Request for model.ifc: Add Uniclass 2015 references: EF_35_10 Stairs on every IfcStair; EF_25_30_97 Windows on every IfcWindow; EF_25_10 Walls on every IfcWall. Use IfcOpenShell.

First a look at what the model holds.

```python
import ifcopenshell

model = ifcopenshell.open("model.ifc")
print(model.schema)
print("classifications:", [c.Name for c in model.by_type("IfcClassification")])
for ifc_class in ("IfcDoor", "IfcRoof", "IfcStair", "IfcWall", "IfcWindow"):
    print(ifc_class, len(model.by_type(ifc_class)))
```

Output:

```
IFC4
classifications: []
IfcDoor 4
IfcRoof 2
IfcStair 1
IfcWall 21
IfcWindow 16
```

```python
import ifcopenshell
import ifcopenshell.api.classification

model = ifcopenshell.open("model.ifc")

system = ifcopenshell.api.classification.add_classification(model, classification="Uniclass 2015")

codes = {
    "IfcStair": ("EF_35_10", "Stairs"),
    "IfcWindow": ("EF_25_30_97", "Windows"),
    "IfcWall": ("EF_25_10", "Walls"),
}
for ifc_class, (code, name) in codes.items():
    products = model.by_type(ifc_class)
    ifcopenshell.api.classification.add_reference(
        model, products=products, classification=system, identification=code, name=name
    )
    print(code, len(products))

model.write("model_updated.ifc")
```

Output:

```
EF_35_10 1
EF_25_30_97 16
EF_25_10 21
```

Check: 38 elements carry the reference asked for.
